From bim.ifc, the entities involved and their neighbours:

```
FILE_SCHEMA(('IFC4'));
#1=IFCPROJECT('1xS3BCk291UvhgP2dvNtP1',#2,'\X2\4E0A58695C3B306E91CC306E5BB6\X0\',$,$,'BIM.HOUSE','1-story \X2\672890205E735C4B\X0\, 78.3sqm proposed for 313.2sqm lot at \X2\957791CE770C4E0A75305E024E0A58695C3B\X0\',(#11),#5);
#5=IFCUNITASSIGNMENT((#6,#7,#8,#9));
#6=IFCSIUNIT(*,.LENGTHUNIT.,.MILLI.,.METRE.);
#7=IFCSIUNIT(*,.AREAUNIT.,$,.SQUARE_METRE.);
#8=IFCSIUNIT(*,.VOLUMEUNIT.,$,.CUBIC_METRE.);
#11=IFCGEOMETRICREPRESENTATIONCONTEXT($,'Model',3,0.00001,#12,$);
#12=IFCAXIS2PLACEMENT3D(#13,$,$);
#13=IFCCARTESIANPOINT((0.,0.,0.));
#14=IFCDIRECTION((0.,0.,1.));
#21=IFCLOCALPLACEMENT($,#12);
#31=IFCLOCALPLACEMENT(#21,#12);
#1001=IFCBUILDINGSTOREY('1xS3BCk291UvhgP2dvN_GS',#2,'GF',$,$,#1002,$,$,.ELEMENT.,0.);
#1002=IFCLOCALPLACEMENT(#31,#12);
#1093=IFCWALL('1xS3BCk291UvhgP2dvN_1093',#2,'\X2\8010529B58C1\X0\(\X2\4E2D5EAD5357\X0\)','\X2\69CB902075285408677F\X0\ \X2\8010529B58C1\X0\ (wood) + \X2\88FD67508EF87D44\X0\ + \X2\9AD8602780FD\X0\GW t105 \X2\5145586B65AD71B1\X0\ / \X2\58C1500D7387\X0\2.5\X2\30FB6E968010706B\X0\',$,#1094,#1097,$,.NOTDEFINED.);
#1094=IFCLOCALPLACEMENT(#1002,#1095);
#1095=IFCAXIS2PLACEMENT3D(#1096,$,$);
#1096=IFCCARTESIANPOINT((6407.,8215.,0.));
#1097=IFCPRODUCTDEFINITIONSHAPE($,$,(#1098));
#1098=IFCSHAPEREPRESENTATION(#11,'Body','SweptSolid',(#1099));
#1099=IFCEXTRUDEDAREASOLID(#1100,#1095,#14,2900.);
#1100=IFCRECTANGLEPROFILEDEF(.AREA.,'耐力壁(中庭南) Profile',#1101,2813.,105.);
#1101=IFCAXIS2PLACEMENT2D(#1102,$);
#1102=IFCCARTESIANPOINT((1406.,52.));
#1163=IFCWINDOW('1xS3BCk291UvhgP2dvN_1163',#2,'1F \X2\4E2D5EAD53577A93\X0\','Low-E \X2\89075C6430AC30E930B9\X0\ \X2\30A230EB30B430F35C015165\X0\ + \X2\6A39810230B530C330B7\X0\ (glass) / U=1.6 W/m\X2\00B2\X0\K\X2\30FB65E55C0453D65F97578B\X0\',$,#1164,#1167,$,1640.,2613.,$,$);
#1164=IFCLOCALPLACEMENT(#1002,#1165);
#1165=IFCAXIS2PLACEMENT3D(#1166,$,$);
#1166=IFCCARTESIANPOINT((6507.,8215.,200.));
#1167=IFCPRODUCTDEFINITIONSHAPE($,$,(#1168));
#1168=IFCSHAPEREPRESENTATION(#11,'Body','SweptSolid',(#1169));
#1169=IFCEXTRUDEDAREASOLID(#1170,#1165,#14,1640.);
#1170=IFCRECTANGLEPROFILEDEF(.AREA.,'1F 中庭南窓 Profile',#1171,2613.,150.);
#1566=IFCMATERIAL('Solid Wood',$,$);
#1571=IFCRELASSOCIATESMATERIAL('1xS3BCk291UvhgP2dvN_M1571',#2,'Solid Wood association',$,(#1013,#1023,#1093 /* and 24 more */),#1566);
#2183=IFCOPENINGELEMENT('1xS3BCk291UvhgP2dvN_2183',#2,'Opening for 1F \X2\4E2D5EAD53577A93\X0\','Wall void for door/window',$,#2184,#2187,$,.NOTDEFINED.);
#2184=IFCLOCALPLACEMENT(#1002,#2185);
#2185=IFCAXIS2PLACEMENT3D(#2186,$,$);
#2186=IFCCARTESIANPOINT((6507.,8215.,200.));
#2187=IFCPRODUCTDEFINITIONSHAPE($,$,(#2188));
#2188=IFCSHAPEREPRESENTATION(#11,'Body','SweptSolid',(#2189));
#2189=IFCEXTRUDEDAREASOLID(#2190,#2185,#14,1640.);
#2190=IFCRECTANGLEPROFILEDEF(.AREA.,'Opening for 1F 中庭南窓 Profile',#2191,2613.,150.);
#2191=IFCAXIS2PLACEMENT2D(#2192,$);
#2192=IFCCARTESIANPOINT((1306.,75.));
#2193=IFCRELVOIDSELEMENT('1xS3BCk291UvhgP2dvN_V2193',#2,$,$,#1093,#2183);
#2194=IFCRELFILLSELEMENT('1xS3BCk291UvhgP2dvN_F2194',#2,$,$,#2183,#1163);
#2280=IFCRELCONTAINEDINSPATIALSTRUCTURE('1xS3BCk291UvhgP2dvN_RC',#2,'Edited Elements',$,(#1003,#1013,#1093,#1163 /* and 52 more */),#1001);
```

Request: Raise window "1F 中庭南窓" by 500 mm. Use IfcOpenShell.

```python
import numpy as np
import ifcopenshell
import ifcopenshell.api.geometry
import ifcopenshell.util.placement
import ifcopenshell.util.unit

model = ifcopenshell.open("bim.ifc")
unit_scale = ifcopenshell.util.unit.calculate_unit_scale(model)

window = model.by_guid("1xS3BCk291UvhgP2dvN_1163")
opening = window.FillsVoids[0].RelatingOpeningElement
dz = 0.5 / unit_scale

shift = np.array([0.0, 0.0, dz])
# The window is not placed relative to its opening, so move both.
for product in (opening, window):
    matrix = ifcopenshell.util.placement.get_local_placement(product.ObjectPlacement)
    matrix[:3, 3] += shift
    ifcopenshell.api.geometry.edit_object_placement(model, product=product, matrix=matrix, is_si=False)

print(f"moved by {dz * unit_scale:+.3f} m")

model.write("bim_v2.ifc")
```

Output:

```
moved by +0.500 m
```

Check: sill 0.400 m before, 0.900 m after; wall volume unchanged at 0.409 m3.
